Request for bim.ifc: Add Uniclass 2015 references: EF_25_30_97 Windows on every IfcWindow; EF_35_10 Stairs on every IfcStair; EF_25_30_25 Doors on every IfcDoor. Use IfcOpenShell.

First a look at what the model holds.

```python
import ifcopenshell

model = ifcopenshell.open("bim.ifc")
print(model.schema)
print("classifications:", [c.Name for c in model.by_type("IfcClassification")])
for ifc_class in ("IfcDoor", "IfcRoof", "IfcStair", "IfcWall", "IfcWindow"):
    print(ifc_class, len(model.by_type(ifc_class)))
```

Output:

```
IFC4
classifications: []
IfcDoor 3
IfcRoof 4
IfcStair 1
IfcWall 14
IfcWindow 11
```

```python
import ifcopenshell
import ifcopenshell.api.classification

model = ifcopenshell.open("bim.ifc")

system = ifcopenshell.api.classification.add_classification(model, classification="Uniclass 2015")

codes = {
    "IfcWindow": ("EF_25_30_97", "Windows"),
    "IfcStair": ("EF_35_10", "Stairs"),
    "IfcDoor": ("EF_25_30_25", "Doors"),
}
for ifc_class, (code, name) in codes.items():
    products = model.by_type(ifc_class)
    ifcopenshell.api.classification.add_reference(
        model, products=products, classification=system, identification=code, name=name
    )
    print(code, len(products))

model.write("bim-out.ifc")
```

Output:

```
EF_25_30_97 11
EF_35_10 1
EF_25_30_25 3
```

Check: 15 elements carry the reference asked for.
